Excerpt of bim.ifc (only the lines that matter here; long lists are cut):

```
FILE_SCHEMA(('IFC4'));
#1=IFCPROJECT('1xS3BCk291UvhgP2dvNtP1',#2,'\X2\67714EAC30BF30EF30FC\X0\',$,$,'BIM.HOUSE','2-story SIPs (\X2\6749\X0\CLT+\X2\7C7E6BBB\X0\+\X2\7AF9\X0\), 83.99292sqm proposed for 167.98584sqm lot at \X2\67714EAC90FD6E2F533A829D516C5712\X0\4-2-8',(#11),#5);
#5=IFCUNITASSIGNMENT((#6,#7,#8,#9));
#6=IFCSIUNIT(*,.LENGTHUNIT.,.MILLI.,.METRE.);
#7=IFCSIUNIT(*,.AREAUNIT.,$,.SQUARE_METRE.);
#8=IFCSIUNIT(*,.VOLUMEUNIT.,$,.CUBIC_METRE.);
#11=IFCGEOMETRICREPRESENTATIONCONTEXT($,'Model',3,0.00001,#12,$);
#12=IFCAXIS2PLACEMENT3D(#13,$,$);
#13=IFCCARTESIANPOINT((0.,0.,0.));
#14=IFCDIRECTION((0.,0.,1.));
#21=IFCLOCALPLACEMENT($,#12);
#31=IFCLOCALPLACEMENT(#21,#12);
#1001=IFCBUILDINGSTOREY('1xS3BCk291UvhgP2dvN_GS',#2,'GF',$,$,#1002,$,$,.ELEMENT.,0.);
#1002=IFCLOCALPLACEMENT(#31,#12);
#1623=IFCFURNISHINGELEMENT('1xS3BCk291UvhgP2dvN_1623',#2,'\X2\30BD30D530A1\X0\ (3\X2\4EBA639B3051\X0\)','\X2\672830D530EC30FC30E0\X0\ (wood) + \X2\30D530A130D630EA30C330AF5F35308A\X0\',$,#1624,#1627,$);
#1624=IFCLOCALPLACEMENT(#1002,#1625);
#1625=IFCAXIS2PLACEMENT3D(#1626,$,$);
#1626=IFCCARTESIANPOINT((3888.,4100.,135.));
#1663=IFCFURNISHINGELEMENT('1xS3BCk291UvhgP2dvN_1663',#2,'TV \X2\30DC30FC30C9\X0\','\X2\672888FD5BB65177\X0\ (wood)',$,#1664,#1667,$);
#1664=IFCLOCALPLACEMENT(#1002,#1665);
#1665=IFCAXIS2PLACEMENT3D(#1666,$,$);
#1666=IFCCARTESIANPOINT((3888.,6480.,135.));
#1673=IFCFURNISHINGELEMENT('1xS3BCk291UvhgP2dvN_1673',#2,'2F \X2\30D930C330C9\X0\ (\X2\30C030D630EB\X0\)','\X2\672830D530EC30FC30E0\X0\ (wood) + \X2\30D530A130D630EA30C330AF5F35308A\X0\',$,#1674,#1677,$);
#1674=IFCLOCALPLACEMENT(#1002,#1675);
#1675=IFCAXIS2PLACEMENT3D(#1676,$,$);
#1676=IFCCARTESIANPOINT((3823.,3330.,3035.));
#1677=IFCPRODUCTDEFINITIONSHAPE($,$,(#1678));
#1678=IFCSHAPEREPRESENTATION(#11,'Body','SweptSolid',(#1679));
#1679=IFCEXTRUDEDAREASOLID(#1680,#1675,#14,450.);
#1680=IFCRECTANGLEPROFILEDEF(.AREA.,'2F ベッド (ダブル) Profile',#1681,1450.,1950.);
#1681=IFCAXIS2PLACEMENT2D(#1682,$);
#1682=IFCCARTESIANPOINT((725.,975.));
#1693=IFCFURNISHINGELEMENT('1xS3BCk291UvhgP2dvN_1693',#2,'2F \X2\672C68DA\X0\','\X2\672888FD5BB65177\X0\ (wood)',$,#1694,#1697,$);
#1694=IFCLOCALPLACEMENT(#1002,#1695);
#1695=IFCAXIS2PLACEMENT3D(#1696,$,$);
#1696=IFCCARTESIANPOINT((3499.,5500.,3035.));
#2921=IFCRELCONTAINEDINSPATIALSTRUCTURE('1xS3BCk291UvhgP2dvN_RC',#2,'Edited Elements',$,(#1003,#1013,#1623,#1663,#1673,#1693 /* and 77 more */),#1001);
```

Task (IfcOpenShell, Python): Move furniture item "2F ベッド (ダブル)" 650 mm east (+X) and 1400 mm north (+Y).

```python
import ifcopenshell
import ifcopenshell.api.geometry
import ifcopenshell.util.placement

model = ifcopenshell.open("bim.ifc")

item = model.by_guid("1xS3BCk291UvhgP2dvN_1673")
matrix = ifcopenshell.util.placement.get_local_placement(item.ObjectPlacement)
matrix[0, 3] += 650.0
matrix[1, 3] += 1400.0
ifcopenshell.api.geometry.edit_object_placement(model, product=item, matrix=matrix, is_si=False)

print(ifcopenshell.util.placement.get_local_placement(item.ObjectPlacement).round(3) + 0.0)

model.write("bim_updated.ifc")
```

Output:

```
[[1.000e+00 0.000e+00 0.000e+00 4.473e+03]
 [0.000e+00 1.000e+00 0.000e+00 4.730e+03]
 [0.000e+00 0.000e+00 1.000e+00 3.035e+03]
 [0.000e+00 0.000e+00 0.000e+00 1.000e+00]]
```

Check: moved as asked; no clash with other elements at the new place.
